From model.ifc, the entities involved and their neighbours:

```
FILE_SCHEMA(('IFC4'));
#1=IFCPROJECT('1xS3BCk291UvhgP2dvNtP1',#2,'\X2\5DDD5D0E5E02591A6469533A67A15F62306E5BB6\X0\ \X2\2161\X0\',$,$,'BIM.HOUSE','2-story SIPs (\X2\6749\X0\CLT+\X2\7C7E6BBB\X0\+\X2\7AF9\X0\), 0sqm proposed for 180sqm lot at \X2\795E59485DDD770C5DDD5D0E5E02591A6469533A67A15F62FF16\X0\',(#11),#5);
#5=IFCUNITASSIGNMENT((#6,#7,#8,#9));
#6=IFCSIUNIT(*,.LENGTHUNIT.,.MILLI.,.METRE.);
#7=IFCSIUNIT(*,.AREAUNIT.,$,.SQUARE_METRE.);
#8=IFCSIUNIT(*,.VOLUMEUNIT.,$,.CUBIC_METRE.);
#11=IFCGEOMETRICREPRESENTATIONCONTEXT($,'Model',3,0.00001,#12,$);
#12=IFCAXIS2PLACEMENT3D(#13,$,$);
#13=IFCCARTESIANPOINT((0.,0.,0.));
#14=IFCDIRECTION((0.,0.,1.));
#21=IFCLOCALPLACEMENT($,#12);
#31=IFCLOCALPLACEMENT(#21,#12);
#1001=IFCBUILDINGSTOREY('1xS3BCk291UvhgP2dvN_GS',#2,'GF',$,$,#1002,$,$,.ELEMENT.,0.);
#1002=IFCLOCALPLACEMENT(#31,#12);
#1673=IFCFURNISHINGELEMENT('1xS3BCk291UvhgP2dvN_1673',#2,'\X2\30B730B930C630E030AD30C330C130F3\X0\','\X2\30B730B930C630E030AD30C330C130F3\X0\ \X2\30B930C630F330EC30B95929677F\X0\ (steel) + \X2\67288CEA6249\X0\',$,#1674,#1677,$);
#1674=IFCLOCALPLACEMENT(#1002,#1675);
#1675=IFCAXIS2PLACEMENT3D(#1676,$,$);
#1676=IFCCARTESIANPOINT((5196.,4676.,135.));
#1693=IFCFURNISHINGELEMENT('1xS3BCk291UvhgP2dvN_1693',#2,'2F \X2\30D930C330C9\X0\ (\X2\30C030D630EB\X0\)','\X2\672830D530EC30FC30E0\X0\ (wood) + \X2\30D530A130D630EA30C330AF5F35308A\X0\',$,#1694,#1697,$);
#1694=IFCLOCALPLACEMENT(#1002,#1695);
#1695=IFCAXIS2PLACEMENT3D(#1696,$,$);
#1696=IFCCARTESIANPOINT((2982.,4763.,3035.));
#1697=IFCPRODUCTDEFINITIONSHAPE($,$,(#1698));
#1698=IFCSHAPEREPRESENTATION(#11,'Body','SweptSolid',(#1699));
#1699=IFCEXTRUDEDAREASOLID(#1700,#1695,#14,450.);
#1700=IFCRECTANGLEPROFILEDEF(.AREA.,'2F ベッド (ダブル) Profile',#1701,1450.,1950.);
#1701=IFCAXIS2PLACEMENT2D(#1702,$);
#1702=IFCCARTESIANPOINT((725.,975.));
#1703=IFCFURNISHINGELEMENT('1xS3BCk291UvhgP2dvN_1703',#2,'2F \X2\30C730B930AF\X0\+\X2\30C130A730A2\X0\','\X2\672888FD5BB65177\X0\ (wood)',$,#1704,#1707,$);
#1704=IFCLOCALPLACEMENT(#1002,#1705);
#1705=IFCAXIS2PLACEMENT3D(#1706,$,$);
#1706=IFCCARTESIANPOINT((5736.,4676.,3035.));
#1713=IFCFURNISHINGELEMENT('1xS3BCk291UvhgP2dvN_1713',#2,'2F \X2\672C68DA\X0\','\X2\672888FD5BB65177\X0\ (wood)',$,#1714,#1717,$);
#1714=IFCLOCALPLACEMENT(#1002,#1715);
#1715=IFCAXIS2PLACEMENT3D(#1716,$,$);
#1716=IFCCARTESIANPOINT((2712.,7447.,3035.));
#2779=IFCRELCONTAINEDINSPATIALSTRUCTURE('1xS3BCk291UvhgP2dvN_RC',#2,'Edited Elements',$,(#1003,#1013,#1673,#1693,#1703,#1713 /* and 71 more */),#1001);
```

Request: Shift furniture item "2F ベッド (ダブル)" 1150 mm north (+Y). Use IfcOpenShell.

```python
import ifcopenshell
import ifcopenshell.api.geometry
import ifcopenshell.util.placement

model = ifcopenshell.open("model.ifc")

item = model.by_guid("1xS3BCk291UvhgP2dvN_1693")
matrix = ifcopenshell.util.placement.get_local_placement(item.ObjectPlacement)
matrix[1, 3] += 1150.0
ifcopenshell.api.geometry.edit_object_placement(model, product=item, matrix=matrix, is_si=False)

print(ifcopenshell.util.placement.get_local_placement(item.ObjectPlacement).round(3) + 0.0)

model.write("model_v2.ifc")
```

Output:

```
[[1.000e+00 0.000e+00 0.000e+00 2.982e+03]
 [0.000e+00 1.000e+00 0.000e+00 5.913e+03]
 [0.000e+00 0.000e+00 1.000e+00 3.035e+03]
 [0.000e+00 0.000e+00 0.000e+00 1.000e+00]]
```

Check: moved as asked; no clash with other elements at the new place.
